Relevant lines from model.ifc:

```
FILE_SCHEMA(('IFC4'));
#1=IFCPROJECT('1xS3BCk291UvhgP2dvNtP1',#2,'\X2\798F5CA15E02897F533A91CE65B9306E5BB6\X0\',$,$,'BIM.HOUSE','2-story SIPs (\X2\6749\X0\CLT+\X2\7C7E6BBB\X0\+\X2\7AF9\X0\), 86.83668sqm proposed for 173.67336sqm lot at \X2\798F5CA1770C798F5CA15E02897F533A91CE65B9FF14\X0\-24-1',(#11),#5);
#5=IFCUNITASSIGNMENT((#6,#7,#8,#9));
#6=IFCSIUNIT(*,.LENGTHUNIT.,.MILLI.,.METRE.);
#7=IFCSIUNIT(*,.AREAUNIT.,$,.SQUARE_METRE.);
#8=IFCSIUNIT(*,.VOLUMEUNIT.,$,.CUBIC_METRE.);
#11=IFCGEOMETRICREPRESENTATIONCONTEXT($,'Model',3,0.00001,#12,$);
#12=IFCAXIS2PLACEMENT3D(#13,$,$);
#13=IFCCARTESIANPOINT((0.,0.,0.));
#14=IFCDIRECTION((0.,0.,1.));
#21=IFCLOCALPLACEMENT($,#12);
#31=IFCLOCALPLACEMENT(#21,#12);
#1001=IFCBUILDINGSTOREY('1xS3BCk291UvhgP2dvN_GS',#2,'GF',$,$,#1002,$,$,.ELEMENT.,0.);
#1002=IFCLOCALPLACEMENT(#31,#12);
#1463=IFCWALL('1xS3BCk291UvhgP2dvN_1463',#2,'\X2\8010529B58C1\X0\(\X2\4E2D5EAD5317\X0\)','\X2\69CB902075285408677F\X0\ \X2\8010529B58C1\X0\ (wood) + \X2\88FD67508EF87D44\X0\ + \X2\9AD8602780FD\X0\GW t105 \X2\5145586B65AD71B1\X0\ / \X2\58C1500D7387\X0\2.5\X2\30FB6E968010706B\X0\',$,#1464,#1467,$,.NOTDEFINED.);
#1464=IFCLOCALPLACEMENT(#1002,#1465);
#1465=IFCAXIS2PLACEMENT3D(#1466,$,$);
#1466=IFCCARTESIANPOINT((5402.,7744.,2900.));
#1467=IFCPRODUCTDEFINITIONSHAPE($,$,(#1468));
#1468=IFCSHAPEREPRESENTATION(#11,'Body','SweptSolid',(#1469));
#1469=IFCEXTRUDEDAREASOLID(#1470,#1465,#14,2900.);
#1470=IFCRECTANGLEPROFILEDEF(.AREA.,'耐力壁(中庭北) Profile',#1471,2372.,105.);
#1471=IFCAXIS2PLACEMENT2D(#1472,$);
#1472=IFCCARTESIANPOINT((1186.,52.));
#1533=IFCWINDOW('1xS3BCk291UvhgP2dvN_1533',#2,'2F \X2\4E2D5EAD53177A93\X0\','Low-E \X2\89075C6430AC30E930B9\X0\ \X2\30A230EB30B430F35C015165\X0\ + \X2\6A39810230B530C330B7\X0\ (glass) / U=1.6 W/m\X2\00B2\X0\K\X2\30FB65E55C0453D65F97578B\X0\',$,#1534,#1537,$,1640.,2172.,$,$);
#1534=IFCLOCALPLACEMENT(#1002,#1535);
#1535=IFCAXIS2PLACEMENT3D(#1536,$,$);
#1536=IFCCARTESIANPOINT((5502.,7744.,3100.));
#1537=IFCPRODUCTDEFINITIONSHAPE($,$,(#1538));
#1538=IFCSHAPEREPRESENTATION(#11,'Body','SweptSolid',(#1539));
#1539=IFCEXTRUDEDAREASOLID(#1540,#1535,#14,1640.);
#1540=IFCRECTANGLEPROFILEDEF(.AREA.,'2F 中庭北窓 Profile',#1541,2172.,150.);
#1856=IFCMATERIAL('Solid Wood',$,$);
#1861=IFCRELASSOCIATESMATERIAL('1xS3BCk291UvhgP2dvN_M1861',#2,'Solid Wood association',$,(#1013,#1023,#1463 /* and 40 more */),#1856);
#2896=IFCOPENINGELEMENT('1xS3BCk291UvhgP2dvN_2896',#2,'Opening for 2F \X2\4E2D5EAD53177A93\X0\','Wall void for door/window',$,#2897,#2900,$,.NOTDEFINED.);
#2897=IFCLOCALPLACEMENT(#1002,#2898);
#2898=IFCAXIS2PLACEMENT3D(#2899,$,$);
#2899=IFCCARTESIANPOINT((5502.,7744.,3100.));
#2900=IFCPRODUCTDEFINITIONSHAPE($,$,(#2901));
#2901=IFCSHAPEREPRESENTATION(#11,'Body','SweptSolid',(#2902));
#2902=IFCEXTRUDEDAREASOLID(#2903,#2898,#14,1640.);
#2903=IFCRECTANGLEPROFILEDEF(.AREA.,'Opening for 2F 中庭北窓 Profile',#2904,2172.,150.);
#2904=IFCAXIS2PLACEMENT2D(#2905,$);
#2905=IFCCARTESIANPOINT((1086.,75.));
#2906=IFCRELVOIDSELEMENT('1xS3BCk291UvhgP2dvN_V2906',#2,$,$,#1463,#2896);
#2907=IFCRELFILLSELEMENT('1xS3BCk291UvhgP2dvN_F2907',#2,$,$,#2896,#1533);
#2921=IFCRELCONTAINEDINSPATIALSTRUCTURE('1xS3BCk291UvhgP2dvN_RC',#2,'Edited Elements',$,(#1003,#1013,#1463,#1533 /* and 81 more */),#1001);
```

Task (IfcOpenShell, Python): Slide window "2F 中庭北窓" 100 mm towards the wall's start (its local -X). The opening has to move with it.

```python
import ifcopenshell
import ifcopenshell.api.geometry
import ifcopenshell.util.placement
import ifcopenshell.util.unit

model = ifcopenshell.open("model.ifc")
unit_scale = ifcopenshell.util.unit.calculate_unit_scale(model)

window = model.by_guid("1xS3BCk291UvhgP2dvN_1533")
opening = window.FillsVoids[0].RelatingOpeningElement
wall = opening.VoidsElements[0].RelatingBuildingElement

wall_matrix = ifcopenshell.util.placement.get_local_placement(wall.ObjectPlacement)
shift = wall_matrix[:3, 0] * -0.1 / unit_scale
before = ifcopenshell.util.placement.get_local_placement(window.ObjectPlacement)[:3, 3].copy()

# The window is not placed relative to its opening, so move both.
for product in (opening, window):
    matrix = ifcopenshell.util.placement.get_local_placement(product.ObjectPlacement)
    matrix[:3, 3] += shift
    ifcopenshell.api.geometry.edit_object_placement(model, product=product, matrix=matrix, is_si=False)

after = ifcopenshell.util.placement.get_local_placement(window.ObjectPlacement)[:3, 3]
print("window moved by", (after - before).round(3) + 0.0)

model.write("model-out.ifc")
```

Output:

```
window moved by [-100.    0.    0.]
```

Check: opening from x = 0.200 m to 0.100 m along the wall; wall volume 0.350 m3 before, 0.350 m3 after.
